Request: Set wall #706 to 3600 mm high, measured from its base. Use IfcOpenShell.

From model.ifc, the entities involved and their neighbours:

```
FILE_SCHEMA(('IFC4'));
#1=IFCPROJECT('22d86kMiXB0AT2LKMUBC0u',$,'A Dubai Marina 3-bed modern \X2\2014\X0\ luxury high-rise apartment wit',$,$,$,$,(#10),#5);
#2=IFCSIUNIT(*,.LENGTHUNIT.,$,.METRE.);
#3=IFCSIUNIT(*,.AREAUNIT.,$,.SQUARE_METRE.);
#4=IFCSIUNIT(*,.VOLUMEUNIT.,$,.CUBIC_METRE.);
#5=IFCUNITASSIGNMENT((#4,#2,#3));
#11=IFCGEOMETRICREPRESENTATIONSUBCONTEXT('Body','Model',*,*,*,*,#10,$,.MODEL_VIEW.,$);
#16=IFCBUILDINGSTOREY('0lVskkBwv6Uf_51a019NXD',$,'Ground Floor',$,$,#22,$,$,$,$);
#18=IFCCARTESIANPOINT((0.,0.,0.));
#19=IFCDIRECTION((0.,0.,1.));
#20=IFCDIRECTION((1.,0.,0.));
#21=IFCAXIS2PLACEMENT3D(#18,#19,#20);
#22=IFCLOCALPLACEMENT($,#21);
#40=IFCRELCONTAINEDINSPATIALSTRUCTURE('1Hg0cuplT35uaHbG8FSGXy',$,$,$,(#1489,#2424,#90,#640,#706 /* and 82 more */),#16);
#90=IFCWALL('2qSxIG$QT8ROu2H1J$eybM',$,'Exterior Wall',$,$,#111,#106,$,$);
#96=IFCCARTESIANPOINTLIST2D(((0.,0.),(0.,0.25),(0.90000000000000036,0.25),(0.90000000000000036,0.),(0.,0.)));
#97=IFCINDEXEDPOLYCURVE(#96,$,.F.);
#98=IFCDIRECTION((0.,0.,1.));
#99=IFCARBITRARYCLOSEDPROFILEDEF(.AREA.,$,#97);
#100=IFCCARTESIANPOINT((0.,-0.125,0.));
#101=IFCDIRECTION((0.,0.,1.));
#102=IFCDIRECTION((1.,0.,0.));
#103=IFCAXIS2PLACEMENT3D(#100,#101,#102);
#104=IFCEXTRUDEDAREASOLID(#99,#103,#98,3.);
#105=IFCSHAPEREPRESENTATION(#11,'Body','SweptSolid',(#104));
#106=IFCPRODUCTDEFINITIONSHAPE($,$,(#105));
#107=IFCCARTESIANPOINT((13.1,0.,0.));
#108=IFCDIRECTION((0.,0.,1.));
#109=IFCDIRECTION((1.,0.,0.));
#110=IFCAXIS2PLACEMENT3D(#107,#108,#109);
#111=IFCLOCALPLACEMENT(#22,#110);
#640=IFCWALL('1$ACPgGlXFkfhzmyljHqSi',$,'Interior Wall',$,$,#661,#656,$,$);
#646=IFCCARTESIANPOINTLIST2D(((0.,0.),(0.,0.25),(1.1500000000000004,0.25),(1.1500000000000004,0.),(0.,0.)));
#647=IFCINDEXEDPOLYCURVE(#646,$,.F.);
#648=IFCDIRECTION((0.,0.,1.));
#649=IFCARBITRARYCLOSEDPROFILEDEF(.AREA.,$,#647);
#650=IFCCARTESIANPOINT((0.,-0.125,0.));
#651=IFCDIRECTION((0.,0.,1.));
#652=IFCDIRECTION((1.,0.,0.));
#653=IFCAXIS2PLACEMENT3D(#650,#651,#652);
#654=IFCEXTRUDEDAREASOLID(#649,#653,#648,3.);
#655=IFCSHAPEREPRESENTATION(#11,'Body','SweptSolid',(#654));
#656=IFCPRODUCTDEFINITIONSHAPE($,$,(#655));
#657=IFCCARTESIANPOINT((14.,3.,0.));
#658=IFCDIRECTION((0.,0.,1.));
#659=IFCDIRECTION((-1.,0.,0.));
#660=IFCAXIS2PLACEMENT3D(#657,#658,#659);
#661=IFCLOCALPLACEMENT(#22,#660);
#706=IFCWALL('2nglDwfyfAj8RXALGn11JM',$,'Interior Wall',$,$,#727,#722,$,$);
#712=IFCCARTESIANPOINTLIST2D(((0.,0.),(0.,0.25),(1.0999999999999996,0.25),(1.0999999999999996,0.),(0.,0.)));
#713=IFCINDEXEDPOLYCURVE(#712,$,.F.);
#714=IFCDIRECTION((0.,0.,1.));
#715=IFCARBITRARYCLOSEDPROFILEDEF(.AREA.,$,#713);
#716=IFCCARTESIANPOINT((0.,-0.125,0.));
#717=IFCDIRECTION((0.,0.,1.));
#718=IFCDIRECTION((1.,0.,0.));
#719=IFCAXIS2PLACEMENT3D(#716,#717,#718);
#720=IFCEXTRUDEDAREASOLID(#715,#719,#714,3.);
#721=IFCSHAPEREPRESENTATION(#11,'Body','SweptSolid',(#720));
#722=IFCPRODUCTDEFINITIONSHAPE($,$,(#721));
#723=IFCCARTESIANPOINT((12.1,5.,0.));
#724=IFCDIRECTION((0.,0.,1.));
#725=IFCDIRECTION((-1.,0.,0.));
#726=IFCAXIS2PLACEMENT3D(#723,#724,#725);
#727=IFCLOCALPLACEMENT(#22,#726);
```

```python
import ifcopenshell
import ifcopenshell.geom
import ifcopenshell.util.representation
import ifcopenshell.util.shape

model = ifcopenshell.open("model.ifc")
settings = ifcopenshell.geom.settings()


def volume(element):
    """Net volume in cubic metres, openings subtracted."""
    shape = ifcopenshell.geom.create_shape(settings, element)
    return ifcopenshell.util.shape.get_volume(shape.geometry)


wall = model.by_guid("2nglDwfyfAj8RXALGn11JM")
before = volume(wall)

body = ifcopenshell.util.representation.get_representation(wall, "Model", "Body")
solid = body.Items[0]
old_height = solid.Depth
solid.Depth = 3.6
after = volume(wall)

print(f"height {old_height:g} -> {solid.Depth:g}, volume {before:.3f} -> {after:.3f} m3")

model.write("model_edited.ifc")
```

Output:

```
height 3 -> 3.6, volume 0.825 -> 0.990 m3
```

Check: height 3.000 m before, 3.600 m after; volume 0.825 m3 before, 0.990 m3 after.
